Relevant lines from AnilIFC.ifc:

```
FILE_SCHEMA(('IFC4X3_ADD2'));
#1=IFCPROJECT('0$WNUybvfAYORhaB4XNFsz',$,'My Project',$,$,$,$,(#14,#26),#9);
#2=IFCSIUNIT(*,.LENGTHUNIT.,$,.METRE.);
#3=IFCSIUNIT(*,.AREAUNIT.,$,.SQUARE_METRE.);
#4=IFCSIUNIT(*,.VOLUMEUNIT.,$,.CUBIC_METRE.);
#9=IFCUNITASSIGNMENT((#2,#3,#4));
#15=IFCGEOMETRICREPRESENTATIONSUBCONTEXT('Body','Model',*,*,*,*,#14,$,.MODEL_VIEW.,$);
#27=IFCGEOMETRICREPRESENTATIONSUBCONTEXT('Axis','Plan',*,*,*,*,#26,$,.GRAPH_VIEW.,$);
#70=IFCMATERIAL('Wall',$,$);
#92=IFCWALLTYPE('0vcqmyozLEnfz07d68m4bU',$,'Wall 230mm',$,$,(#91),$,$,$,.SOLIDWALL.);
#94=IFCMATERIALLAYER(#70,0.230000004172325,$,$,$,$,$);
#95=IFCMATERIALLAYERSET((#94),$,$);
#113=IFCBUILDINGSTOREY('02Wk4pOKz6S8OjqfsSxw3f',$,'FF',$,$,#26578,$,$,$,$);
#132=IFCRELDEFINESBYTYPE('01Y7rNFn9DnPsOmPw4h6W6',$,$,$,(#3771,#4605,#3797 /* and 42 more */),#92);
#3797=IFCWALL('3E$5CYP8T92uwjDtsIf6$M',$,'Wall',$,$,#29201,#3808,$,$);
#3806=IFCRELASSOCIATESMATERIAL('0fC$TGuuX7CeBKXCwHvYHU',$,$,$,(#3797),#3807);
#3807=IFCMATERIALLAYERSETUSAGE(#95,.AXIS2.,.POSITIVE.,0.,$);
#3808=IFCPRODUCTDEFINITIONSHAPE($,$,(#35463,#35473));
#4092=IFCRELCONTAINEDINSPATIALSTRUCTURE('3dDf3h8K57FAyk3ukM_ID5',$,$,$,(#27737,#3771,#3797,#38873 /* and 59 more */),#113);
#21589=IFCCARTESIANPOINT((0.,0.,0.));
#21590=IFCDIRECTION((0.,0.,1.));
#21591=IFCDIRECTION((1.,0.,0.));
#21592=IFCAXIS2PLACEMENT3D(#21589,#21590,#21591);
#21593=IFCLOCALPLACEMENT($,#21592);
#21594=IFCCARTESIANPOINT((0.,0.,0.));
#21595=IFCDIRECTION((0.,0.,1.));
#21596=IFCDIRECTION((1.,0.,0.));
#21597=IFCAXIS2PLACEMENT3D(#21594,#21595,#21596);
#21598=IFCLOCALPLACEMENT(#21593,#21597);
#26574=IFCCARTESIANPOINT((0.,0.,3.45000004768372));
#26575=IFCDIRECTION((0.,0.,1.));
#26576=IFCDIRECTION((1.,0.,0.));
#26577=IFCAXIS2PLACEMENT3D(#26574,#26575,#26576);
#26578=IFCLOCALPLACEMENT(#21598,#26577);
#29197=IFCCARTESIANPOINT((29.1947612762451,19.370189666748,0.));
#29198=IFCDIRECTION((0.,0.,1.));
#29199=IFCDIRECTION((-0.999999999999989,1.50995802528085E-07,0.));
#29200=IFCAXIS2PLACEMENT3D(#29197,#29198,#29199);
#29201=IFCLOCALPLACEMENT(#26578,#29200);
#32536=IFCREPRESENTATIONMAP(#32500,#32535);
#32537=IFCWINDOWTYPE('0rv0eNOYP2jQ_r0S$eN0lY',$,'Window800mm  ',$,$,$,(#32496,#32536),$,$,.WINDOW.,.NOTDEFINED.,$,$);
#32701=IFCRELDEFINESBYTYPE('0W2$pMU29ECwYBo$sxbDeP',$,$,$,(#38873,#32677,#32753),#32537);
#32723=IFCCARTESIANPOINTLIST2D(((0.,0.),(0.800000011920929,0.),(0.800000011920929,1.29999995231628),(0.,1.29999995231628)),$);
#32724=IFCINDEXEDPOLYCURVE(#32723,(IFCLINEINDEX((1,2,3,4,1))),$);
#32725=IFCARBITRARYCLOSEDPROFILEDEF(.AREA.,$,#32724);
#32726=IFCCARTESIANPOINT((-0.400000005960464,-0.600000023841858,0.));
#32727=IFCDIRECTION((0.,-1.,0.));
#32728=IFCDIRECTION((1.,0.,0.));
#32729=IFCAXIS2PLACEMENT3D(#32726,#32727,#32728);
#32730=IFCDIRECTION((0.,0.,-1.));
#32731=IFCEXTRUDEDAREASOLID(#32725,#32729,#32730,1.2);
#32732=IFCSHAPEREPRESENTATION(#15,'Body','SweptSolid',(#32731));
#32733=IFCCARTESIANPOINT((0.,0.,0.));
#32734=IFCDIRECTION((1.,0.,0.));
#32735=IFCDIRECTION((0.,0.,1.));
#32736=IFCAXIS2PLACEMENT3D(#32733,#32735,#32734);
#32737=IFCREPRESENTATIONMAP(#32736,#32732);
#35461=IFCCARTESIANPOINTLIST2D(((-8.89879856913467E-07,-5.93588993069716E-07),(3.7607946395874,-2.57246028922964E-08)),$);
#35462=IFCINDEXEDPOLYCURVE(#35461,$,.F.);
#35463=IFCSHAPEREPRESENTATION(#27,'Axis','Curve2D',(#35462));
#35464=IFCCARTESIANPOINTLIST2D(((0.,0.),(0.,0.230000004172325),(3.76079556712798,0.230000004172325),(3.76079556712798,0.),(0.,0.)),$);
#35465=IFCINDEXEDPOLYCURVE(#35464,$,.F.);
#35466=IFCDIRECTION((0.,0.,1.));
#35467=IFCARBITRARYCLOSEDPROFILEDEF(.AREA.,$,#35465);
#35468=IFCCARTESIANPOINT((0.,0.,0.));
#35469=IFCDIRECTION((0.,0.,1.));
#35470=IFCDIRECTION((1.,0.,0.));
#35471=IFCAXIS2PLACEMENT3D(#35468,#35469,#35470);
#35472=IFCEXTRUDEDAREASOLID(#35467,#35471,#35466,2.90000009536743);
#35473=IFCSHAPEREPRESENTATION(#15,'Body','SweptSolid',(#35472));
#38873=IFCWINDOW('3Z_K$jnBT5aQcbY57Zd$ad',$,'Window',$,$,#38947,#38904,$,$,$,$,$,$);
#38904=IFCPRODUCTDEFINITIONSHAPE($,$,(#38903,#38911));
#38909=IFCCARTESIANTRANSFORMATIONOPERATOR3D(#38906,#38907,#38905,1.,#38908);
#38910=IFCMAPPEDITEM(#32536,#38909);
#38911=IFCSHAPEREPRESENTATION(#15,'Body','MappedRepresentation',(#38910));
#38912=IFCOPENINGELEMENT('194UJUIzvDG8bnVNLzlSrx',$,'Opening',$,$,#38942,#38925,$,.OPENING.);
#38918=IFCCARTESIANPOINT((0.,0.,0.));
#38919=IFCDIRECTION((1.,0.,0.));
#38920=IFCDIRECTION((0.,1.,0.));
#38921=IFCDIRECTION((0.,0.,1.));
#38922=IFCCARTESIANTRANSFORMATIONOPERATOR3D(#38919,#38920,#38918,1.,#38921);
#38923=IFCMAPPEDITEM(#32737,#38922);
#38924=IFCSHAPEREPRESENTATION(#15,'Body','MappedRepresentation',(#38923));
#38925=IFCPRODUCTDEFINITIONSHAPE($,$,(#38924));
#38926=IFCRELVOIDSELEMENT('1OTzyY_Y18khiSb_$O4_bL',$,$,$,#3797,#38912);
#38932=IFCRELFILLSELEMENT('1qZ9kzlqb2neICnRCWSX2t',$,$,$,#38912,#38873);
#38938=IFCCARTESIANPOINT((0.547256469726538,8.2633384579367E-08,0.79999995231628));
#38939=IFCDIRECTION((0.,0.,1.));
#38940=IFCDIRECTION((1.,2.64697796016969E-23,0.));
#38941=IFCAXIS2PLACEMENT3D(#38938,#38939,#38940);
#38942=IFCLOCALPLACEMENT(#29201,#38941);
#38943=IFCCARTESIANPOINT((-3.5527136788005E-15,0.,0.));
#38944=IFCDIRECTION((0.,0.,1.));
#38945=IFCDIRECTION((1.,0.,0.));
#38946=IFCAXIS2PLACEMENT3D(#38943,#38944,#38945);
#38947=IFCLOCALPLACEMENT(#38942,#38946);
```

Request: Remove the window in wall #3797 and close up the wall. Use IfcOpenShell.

```python
import ifcopenshell
import ifcopenshell.api.feature
import ifcopenshell.api.root
import ifcopenshell.geom
import ifcopenshell.util.shape

model = ifcopenshell.open("AnilIFC.ifc")
settings = ifcopenshell.geom.settings()


def volume(element):
    """Net volume in cubic metres, openings subtracted."""
    shape = ifcopenshell.geom.create_shape(settings, element)
    return ifcopenshell.util.shape.get_volume(shape.geometry)


window = model.by_guid("3Z_K$jnBT5aQcbY57Zd$ad")
opening = window.FillsVoids[0].RelatingOpeningElement
wall = opening.VoidsElements[0].RelatingBuildingElement
before = volume(wall)

ifcopenshell.api.root.remove_product(model, product=window)
ifcopenshell.api.feature.remove_feature(model, feature=opening)

after = volume(wall)

print(f"wall volume {before:.3f} -> {after:.3f} m3")

model.write("AnilIFC_v2.ifc")
```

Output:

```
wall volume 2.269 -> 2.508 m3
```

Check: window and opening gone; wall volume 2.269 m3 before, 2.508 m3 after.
